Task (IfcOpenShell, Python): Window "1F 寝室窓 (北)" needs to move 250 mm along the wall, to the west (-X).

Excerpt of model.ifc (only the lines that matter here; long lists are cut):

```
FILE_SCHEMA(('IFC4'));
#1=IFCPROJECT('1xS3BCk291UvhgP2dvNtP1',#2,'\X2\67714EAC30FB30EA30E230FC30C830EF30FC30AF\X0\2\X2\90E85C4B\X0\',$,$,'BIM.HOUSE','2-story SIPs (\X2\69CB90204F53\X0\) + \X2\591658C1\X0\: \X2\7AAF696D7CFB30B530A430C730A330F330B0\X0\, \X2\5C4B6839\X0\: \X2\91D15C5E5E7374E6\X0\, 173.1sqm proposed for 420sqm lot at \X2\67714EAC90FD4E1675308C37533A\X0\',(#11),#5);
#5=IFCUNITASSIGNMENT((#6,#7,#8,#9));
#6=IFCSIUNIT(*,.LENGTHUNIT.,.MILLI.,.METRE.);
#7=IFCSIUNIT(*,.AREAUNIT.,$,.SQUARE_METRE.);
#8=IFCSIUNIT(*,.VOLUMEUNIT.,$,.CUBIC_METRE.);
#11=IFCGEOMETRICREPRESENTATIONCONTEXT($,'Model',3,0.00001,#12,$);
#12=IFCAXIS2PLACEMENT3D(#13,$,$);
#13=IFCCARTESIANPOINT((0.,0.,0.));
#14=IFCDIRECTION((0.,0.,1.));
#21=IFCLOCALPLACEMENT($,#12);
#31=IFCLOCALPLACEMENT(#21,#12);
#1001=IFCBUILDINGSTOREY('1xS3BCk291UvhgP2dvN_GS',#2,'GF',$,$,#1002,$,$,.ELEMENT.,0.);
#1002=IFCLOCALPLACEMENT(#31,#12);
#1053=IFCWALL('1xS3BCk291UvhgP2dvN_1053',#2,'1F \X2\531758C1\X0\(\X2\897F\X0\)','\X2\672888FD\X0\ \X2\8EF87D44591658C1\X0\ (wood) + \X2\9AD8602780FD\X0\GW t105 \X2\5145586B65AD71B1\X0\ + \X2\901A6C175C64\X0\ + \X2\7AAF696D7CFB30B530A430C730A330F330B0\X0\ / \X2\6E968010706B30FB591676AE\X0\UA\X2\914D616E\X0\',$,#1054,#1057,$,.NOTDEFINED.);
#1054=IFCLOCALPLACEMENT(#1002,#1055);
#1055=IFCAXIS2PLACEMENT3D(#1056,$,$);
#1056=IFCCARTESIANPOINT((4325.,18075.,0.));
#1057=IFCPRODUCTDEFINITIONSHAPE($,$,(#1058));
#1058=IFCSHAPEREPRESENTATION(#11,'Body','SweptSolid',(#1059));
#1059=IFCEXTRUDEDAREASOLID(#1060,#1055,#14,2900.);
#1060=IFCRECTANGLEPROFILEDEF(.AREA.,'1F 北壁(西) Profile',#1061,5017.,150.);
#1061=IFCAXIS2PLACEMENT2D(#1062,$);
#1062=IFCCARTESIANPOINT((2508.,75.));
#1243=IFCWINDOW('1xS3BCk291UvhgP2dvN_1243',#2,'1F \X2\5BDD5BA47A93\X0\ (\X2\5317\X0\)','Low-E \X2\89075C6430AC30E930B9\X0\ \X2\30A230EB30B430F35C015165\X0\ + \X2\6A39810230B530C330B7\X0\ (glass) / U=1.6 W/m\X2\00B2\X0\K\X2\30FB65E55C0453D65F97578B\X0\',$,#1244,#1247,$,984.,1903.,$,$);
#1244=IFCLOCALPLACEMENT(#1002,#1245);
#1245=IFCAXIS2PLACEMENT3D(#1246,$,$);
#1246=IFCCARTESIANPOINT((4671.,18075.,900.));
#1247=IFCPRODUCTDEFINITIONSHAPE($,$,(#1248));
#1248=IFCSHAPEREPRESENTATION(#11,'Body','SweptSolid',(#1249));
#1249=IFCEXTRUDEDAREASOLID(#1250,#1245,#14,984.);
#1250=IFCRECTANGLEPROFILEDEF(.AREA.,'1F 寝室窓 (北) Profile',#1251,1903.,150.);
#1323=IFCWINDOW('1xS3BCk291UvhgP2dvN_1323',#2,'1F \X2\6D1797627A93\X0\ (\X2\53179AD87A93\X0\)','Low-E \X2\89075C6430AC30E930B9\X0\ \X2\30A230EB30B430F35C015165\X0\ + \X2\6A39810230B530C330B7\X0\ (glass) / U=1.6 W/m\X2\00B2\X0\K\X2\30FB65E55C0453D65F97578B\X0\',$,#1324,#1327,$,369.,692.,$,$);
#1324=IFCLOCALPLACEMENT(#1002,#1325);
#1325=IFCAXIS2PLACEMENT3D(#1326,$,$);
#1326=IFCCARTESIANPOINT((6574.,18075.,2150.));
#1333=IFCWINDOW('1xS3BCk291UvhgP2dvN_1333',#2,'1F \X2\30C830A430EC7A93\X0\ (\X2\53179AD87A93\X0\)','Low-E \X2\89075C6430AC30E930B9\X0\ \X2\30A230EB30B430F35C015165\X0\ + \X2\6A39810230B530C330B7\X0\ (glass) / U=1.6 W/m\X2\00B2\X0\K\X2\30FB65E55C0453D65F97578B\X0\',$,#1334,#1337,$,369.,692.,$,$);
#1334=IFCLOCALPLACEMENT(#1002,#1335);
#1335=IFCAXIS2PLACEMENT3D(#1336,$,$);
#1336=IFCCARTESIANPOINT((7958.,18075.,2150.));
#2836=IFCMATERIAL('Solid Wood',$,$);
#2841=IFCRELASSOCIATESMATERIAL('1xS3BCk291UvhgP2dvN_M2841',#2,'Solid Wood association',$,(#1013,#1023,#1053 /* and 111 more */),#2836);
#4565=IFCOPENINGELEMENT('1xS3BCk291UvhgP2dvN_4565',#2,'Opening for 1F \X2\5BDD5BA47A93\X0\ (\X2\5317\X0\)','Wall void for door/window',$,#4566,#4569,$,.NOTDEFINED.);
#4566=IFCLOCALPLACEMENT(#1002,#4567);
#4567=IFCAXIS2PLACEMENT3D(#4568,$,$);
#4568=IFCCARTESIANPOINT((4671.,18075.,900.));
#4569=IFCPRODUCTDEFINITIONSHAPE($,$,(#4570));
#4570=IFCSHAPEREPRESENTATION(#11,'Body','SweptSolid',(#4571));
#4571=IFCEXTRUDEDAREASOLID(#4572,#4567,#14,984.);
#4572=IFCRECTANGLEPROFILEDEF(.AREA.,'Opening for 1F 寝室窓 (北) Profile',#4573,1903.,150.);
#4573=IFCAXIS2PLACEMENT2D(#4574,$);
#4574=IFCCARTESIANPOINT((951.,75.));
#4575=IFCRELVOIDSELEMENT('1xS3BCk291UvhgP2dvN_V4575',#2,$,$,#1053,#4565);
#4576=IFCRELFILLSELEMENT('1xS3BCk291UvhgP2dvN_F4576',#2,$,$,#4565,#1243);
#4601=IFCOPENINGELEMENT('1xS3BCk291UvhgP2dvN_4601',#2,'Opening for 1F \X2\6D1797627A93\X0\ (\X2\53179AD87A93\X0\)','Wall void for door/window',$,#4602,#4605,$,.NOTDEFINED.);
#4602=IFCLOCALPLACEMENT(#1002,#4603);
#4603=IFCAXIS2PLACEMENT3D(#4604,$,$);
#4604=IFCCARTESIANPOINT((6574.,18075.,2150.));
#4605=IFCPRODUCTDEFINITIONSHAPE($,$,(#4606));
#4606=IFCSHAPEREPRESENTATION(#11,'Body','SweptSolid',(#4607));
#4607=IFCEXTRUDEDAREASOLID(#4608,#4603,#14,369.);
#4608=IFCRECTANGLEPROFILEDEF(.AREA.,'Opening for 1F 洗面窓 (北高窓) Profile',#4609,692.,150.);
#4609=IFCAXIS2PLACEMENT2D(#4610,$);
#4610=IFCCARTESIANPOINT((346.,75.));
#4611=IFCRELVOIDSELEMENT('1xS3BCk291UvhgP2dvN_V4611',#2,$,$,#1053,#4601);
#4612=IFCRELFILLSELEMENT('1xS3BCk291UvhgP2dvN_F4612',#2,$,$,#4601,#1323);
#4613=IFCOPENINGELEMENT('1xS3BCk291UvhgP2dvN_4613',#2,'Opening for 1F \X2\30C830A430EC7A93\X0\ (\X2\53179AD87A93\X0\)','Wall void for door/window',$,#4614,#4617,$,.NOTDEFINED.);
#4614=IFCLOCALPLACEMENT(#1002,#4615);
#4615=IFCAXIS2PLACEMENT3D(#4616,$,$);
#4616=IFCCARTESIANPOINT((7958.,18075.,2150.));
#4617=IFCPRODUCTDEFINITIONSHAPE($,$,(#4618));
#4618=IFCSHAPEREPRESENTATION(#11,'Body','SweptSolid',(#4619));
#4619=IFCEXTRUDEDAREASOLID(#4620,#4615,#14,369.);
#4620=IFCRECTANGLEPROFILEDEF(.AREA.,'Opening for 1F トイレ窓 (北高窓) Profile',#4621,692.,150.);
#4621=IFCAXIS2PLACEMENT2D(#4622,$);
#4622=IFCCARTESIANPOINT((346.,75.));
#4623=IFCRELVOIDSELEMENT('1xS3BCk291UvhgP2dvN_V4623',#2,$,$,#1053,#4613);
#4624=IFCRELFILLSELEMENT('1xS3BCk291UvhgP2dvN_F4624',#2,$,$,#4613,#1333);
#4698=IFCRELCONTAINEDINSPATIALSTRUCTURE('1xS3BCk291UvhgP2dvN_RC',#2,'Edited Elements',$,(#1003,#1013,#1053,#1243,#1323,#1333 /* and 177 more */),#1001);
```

```python
import ifcopenshell
import ifcopenshell.api.geometry
import ifcopenshell.util.placement
import ifcopenshell.util.unit

model = ifcopenshell.open("model.ifc")
unit_scale = ifcopenshell.util.unit.calculate_unit_scale(model)

window = model.by_guid("1xS3BCk291UvhgP2dvN_1243")
opening = window.FillsVoids[0].RelatingOpeningElement
wall = opening.VoidsElements[0].RelatingBuildingElement

wall_matrix = ifcopenshell.util.placement.get_local_placement(wall.ObjectPlacement)
shift = wall_matrix[:3, 0] * -0.25 / unit_scale
before = ifcopenshell.util.placement.get_local_placement(window.ObjectPlacement)[:3, 3].copy()

# The window is not placed relative to its opening, so move both.
for product in (opening, window):
    matrix = ifcopenshell.util.placement.get_local_placement(product.ObjectPlacement)
    matrix[:3, 3] += shift
    ifcopenshell.api.geometry.edit_object_placement(model, product=product, matrix=matrix, is_si=False)

after = ifcopenshell.util.placement.get_local_placement(window.ObjectPlacement)[:3, 3]
print("window moved by", (after - before).round(3) + 0.0)

model.write("model_v2.ifc")
```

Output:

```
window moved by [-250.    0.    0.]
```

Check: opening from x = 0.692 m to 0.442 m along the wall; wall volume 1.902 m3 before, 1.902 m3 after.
